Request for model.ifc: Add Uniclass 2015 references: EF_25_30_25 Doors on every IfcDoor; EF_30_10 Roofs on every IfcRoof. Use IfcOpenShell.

First a look at what the model holds.

```python
import ifcopenshell

model = ifcopenshell.open("model.ifc")
print(model.schema)
print("classifications:", [c.Name for c in model.by_type("IfcClassification")])
for ifc_class in ("IfcDoor", "IfcRoof", "IfcStair", "IfcWall", "IfcWindow"):
    print(ifc_class, len(model.by_type(ifc_class)))
```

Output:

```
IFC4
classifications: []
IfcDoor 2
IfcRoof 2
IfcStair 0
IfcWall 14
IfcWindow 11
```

```python
import ifcopenshell
import ifcopenshell.api.classification

model = ifcopenshell.open("model.ifc")

system = ifcopenshell.api.classification.add_classification(model, classification="Uniclass 2015")

codes = {
    "IfcDoor": ("EF_25_30_25", "Doors"),
    "IfcRoof": ("EF_30_10", "Roofs"),
}
for ifc_class, (code, name) in codes.items():
    products = model.by_type(ifc_class)
    ifcopenshell.api.classification.add_reference(
        model, products=products, classification=system, identification=code, name=name
    )
    print(code, len(products))

model.write("model-out.ifc")
```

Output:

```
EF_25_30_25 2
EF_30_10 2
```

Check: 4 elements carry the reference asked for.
